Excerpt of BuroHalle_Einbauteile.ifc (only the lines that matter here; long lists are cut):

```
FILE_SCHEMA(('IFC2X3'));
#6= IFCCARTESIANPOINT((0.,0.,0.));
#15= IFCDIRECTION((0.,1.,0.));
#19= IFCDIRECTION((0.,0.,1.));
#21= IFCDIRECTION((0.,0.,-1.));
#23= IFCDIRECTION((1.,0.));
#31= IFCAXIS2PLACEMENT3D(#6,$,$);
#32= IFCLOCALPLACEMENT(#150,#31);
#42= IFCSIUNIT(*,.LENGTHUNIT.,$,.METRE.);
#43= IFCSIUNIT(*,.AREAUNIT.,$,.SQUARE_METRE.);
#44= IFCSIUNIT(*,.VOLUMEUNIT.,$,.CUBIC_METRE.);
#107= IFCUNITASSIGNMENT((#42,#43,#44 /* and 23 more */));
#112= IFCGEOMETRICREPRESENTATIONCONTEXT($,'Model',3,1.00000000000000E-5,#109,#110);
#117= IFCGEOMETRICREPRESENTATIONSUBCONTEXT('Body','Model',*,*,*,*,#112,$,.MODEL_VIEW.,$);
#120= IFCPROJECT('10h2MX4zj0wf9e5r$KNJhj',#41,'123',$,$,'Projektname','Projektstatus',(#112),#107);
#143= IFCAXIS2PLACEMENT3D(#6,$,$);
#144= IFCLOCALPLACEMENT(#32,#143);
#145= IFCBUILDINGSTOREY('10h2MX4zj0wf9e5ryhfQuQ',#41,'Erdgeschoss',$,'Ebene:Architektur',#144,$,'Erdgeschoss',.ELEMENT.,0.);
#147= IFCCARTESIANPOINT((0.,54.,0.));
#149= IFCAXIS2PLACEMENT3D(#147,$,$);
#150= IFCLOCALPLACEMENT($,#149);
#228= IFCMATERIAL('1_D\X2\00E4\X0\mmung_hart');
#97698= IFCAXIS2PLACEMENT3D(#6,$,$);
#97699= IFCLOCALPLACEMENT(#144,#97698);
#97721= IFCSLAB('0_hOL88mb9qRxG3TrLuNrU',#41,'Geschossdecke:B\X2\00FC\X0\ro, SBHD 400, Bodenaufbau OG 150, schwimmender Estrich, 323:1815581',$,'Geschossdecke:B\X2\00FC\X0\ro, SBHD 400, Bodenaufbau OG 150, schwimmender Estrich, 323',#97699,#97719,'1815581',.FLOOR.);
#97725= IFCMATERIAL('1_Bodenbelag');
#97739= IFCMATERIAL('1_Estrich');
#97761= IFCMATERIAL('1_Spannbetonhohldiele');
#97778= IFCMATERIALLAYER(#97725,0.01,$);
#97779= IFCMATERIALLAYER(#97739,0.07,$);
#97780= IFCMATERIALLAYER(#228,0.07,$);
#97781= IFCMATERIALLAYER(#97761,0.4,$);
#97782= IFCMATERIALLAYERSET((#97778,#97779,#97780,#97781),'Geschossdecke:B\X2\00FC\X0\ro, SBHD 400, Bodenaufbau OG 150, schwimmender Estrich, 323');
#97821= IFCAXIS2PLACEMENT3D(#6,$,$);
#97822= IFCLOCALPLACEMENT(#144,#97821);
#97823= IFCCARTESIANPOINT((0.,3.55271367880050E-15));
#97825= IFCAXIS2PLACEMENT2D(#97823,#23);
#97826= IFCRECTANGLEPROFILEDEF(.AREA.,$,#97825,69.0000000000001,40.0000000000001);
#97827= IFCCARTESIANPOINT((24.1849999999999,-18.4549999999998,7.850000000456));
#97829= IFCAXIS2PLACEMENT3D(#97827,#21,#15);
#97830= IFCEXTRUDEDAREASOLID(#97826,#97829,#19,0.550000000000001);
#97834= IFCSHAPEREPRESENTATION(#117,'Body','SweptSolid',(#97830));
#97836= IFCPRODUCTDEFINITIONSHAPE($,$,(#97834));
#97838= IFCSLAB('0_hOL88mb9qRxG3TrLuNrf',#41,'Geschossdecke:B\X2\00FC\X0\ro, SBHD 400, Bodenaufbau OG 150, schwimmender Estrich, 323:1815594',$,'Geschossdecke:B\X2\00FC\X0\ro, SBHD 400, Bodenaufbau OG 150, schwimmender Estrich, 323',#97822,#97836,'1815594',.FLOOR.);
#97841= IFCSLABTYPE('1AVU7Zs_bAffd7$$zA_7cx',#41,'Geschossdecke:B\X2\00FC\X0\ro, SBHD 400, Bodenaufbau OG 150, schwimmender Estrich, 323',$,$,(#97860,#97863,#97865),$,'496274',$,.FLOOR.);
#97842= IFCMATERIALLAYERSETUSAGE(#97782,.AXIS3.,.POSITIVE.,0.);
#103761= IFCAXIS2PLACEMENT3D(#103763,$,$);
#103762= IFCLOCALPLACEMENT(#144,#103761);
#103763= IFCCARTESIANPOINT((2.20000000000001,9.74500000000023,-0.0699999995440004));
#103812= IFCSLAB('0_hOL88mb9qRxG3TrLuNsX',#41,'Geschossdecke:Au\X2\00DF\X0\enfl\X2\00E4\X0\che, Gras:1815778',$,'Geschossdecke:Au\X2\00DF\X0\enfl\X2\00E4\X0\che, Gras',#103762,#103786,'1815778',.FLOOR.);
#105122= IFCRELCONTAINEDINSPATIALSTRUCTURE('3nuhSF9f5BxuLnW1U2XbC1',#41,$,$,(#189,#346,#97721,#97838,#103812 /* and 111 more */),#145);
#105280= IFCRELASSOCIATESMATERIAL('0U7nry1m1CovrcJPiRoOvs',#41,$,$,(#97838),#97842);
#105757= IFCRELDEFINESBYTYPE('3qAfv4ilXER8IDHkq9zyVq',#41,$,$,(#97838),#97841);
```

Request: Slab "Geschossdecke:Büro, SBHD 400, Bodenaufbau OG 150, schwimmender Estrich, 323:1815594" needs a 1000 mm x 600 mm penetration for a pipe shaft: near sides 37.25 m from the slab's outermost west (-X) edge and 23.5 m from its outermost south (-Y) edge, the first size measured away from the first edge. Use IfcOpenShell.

```python
import numpy as np
import ifcopenshell
import ifcopenshell.api.feature
import ifcopenshell.api.geometry
import ifcopenshell.api.root
import ifcopenshell.geom
import ifcopenshell.util.placement
import ifcopenshell.util.representation
import ifcopenshell.util.shape
import ifcopenshell.util.unit

model = ifcopenshell.open("BuroHalle_Einbauteile.ifc")
unit_scale = ifcopenshell.util.unit.calculate_unit_scale(model)
settings = ifcopenshell.geom.settings()


def volume(element):
    """Net volume in cubic metres, openings subtracted."""
    shape = ifcopenshell.geom.create_shape(settings, element)
    return ifcopenshell.util.shape.get_volume(shape.geometry)


slab = model.by_guid("0_hOL88mb9qRxG3TrLuNrf")
before = volume(slab)

# Extent in the slab's own axes, in metres. The edges named are its -X and -Y sides.
slab_shape = ifcopenshell.geom.create_shape(settings, slab)
vertices = ifcopenshell.util.shape.get_vertices(slab_shape.geometry)
x_min, y_min, bottom = vertices.min(axis=0)
top = vertices[:, 2].max()

opening = ifcopenshell.api.root.create_entity(model, ifc_class="IfcOpeningElement", name="Pipe shaft opening")
context = ifcopenshell.util.representation.get_context(model, "Model", "Body", "MODEL_VIEW")
width, depth = 1, 0.6
outline = [(0.0, 0.0), (width, 0.0), (width, depth), (0.0, depth), (0.0, 0.0)]
# Overshoot both faces by 50 mm so the cut is clean.
shape = ifcopenshell.api.geometry.add_slab_representation(
    model, context=context, depth=top - bottom + 0.1, polyline=outline
)
ifcopenshell.api.geometry.assign_representation(model, product=opening, representation=shape)

matrix = ifcopenshell.util.placement.get_local_placement(slab.ObjectPlacement)
matrix[:, 3] = matrix @ np.append(np.array([x_min + 37.25, y_min + 23.5, bottom - 0.05]) / unit_scale, 1.0)
ifcopenshell.api.geometry.edit_object_placement(model, product=opening, matrix=matrix, is_si=False)
ifcopenshell.api.feature.add_feature(model, feature=opening, element=slab)

after = volume(slab)

print(f"slab volume {before:.3f} -> {after:.3f} m3")

model.write("BuroHalle_Einbauteile_v2.ifc")
```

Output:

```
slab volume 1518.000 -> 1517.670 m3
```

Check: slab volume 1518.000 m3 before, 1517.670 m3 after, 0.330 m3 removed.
